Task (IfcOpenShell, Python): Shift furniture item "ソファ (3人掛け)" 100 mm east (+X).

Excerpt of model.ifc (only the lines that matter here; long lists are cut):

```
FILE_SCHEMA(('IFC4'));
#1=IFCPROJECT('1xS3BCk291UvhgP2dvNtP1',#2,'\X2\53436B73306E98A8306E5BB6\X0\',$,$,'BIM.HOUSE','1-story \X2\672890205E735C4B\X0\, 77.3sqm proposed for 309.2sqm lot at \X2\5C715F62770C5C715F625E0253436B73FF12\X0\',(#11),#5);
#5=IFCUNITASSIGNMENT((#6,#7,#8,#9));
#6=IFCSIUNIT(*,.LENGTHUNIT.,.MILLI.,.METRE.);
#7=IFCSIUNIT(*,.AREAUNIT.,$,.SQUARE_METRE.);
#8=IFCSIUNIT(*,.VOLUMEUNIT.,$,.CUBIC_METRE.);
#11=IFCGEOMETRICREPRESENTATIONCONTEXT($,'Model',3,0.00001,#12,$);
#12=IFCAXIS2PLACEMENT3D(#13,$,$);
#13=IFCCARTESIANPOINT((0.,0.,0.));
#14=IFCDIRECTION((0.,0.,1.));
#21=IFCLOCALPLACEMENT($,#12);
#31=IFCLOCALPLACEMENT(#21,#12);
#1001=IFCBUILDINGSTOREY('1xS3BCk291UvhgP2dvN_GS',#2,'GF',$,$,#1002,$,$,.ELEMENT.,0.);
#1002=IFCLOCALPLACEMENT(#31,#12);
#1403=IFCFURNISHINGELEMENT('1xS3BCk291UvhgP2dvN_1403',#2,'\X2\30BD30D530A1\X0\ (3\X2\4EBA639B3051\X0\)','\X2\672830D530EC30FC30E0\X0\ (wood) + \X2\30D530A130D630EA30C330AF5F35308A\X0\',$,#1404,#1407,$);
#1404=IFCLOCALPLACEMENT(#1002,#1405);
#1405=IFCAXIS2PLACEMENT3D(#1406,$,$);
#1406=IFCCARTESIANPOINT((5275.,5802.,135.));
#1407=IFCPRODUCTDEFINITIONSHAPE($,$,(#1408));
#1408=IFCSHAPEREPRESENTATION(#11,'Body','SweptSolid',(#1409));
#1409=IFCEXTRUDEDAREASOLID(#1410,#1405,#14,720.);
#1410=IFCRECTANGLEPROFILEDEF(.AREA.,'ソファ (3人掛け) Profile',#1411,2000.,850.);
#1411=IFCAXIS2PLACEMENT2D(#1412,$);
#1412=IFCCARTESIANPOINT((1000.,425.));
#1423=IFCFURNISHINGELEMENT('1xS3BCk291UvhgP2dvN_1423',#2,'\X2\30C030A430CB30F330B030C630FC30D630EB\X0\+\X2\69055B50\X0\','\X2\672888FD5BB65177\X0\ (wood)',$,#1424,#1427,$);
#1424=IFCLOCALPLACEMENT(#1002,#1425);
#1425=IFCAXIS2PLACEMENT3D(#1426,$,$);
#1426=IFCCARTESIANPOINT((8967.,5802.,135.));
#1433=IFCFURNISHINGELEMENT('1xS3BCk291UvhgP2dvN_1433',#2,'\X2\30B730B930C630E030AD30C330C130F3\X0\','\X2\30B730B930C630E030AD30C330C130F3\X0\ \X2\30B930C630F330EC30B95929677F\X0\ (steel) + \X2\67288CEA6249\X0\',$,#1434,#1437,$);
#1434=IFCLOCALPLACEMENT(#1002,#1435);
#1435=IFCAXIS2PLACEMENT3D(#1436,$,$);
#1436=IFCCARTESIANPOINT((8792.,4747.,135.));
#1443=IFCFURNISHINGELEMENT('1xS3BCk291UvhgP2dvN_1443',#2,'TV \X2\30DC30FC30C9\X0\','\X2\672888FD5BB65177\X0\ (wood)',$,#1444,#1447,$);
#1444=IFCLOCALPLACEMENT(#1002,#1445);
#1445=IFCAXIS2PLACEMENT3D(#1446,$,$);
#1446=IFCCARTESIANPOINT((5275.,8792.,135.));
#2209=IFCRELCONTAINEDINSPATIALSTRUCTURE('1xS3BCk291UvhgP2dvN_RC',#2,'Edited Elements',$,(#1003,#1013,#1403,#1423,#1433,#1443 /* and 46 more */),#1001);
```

```python
import ifcopenshell
import ifcopenshell.api.geometry
import ifcopenshell.util.placement
import ifcopenshell.util.unit

model = ifcopenshell.open("model.ifc")
unit_scale = ifcopenshell.util.unit.calculate_unit_scale(model)

item = model.by_guid("1xS3BCk291UvhgP2dvN_1403")
matrix = ifcopenshell.util.placement.get_local_placement(item.ObjectPlacement)
matrix[0, 3] += 0.1 / unit_scale
ifcopenshell.api.geometry.edit_object_placement(model, product=item, matrix=matrix, is_si=False)

print(ifcopenshell.util.placement.get_local_placement(item.ObjectPlacement).round(3) + 0.0)

model.write("model_v2.ifc")
```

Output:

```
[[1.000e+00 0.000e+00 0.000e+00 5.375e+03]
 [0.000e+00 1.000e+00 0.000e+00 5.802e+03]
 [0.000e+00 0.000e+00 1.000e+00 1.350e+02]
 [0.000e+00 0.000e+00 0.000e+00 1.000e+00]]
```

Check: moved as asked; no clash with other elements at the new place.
